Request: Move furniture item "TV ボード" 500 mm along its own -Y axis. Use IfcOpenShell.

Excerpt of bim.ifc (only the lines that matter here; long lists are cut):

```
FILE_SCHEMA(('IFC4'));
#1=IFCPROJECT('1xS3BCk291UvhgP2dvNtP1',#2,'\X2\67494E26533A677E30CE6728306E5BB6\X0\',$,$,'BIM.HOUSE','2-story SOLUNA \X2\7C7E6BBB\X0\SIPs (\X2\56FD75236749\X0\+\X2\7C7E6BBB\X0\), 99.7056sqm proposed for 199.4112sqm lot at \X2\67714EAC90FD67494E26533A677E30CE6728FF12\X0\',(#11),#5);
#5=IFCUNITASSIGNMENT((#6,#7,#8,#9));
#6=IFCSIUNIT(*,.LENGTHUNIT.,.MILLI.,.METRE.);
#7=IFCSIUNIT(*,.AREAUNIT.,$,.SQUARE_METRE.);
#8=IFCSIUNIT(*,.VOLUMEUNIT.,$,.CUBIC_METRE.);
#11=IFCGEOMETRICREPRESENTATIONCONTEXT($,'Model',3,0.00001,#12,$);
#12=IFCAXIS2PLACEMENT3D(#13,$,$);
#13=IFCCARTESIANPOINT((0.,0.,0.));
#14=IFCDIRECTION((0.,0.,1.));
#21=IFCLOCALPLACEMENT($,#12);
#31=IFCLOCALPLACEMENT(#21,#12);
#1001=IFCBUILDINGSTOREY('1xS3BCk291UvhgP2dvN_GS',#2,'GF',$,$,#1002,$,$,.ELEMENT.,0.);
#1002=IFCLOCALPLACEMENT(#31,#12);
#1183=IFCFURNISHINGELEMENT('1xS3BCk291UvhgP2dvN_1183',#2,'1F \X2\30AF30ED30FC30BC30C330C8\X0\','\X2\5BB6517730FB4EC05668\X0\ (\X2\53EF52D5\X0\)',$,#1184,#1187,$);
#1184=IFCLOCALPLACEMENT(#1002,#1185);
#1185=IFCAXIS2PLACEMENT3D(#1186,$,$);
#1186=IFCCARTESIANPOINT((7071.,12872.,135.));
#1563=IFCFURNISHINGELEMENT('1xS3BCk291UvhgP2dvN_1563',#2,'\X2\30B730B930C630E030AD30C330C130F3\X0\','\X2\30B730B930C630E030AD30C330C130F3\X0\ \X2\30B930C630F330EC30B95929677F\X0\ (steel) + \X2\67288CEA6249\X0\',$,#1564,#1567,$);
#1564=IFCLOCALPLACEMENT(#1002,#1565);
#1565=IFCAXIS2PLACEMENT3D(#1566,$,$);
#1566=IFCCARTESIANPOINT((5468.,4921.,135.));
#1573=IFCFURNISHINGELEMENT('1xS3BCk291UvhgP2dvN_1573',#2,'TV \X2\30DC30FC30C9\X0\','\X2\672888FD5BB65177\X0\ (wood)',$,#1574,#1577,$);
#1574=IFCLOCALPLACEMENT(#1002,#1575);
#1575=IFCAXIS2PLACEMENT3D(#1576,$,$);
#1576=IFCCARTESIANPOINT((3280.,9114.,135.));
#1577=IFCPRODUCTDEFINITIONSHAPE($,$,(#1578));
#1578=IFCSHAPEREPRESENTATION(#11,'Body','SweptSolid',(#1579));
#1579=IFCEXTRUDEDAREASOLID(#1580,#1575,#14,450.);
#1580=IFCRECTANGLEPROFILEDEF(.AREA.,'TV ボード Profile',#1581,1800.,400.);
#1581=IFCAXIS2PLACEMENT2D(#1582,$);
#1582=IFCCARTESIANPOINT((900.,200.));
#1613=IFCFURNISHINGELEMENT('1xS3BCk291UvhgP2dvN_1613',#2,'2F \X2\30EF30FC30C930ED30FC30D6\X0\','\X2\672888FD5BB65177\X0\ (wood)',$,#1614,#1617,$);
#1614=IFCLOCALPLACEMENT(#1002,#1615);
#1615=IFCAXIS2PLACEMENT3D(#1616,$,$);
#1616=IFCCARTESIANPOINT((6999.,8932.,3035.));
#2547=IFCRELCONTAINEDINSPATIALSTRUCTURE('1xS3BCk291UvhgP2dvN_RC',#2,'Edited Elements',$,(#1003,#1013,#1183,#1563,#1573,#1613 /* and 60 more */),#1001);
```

```python
import ifcopenshell
import ifcopenshell.api.geometry
import ifcopenshell.util.placement
import ifcopenshell.util.unit

model = ifcopenshell.open("bim.ifc")
unit_scale = ifcopenshell.util.unit.calculate_unit_scale(model)

item = model.by_guid("1xS3BCk291UvhgP2dvN_1573")
matrix = ifcopenshell.util.placement.get_local_placement(item.ObjectPlacement)
matrix[:3, 3] -= matrix[:3, 1] * 0.5 / unit_scale
ifcopenshell.api.geometry.edit_object_placement(model, product=item, matrix=matrix, is_si=False)

print(ifcopenshell.util.placement.get_local_placement(item.ObjectPlacement).round(3) + 0.0)

model.write("bim_edited.ifc")
```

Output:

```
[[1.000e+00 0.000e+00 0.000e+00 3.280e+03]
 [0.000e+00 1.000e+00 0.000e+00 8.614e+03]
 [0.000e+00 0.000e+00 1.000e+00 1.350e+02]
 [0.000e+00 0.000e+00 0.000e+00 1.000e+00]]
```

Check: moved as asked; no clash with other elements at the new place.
